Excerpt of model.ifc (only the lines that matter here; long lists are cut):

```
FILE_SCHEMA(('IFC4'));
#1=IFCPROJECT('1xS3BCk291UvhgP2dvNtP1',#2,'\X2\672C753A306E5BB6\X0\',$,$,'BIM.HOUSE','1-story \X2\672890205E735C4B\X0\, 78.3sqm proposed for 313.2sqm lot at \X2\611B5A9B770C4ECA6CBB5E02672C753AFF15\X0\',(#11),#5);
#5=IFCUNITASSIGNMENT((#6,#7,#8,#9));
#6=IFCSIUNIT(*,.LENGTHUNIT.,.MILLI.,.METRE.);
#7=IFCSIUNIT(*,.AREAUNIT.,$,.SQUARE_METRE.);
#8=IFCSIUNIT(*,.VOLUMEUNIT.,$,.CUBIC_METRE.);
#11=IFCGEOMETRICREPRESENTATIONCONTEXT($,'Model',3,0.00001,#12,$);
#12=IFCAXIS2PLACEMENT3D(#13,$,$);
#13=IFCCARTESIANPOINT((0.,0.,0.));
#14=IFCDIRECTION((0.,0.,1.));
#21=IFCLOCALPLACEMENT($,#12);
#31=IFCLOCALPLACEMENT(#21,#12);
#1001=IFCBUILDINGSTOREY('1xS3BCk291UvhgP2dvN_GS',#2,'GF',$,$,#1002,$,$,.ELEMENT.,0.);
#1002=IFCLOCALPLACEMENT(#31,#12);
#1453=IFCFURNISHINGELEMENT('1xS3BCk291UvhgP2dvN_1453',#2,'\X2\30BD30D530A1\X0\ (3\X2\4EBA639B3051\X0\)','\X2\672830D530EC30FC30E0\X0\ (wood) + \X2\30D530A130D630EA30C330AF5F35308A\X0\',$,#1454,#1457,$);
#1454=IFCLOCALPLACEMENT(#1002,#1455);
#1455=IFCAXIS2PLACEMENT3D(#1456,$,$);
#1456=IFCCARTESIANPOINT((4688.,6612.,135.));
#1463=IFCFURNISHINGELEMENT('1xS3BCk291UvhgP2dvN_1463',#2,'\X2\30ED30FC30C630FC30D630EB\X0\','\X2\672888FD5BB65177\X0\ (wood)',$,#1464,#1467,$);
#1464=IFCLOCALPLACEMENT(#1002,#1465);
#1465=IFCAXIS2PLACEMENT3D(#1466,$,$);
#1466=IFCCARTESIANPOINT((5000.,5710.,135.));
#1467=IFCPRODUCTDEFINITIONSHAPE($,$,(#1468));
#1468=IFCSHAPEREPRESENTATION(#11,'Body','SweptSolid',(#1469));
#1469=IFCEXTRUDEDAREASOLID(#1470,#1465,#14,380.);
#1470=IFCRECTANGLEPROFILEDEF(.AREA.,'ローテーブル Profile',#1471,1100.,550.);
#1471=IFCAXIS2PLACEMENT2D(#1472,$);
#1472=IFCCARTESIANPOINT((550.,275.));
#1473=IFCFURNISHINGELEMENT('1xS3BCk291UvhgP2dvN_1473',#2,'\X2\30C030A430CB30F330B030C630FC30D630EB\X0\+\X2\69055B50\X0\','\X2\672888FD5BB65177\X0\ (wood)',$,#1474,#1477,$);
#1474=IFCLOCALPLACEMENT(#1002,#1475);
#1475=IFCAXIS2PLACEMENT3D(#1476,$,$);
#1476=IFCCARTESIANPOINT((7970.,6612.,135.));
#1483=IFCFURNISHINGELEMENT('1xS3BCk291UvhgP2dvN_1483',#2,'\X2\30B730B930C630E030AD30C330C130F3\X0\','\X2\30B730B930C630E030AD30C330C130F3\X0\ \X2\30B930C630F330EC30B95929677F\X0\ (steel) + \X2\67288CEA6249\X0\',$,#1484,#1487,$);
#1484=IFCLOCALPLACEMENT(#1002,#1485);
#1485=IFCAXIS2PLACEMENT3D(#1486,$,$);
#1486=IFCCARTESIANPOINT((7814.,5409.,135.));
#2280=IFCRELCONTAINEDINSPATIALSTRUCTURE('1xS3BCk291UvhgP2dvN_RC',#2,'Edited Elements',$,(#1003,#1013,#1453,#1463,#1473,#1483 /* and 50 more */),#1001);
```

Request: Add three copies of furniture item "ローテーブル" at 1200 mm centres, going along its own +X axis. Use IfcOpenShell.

```python
import ifcopenshell
import ifcopenshell.api.geometry
import ifcopenshell.api.root
import ifcopenshell.util.element
import ifcopenshell.util.placement
import ifcopenshell.util.unit

model = ifcopenshell.open("model.ifc")
unit_scale = ifcopenshell.util.unit.calculate_unit_scale(model)


def reuse_history(source, copy):
    """copy_class also copies each property set's owner history, people and application; keep the originals."""
    for rel in copy.IsDefinedBy:
        if rel.is_a("IfcRelDefinesByProperties") and (history := rel.RelatingPropertyDefinition.OwnerHistory):
            rel.RelatingPropertyDefinition.OwnerHistory = source.OwnerHistory
            ifcopenshell.util.element.remove_deep2(model, history)


source = model.by_guid("1xS3BCk291UvhgP2dvN_1463")
base = ifcopenshell.util.placement.get_local_placement(source.ObjectPlacement)
step = base[:3, 0] * 1.2 / unit_scale

for i in range(1, 4):
    copy = ifcopenshell.api.root.copy_class(model, product=source)
    copy.Representation = ifcopenshell.util.element.copy_deep(
        model, source.Representation, exclude=["IfcGeometricRepresentationContext", "IfcRepresentationMap"]
    )
    reuse_history(source, copy)
    matrix = base.copy()
    matrix[:3, 3] += i * step
    print("added at", matrix[:3, 3].round(3) + 0.0)
    ifcopenshell.api.geometry.edit_object_placement(model, product=copy, matrix=matrix, is_si=False)

model.write("model_v2.ifc")
```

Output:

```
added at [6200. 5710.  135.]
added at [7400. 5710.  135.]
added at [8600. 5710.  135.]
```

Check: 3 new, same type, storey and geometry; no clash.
